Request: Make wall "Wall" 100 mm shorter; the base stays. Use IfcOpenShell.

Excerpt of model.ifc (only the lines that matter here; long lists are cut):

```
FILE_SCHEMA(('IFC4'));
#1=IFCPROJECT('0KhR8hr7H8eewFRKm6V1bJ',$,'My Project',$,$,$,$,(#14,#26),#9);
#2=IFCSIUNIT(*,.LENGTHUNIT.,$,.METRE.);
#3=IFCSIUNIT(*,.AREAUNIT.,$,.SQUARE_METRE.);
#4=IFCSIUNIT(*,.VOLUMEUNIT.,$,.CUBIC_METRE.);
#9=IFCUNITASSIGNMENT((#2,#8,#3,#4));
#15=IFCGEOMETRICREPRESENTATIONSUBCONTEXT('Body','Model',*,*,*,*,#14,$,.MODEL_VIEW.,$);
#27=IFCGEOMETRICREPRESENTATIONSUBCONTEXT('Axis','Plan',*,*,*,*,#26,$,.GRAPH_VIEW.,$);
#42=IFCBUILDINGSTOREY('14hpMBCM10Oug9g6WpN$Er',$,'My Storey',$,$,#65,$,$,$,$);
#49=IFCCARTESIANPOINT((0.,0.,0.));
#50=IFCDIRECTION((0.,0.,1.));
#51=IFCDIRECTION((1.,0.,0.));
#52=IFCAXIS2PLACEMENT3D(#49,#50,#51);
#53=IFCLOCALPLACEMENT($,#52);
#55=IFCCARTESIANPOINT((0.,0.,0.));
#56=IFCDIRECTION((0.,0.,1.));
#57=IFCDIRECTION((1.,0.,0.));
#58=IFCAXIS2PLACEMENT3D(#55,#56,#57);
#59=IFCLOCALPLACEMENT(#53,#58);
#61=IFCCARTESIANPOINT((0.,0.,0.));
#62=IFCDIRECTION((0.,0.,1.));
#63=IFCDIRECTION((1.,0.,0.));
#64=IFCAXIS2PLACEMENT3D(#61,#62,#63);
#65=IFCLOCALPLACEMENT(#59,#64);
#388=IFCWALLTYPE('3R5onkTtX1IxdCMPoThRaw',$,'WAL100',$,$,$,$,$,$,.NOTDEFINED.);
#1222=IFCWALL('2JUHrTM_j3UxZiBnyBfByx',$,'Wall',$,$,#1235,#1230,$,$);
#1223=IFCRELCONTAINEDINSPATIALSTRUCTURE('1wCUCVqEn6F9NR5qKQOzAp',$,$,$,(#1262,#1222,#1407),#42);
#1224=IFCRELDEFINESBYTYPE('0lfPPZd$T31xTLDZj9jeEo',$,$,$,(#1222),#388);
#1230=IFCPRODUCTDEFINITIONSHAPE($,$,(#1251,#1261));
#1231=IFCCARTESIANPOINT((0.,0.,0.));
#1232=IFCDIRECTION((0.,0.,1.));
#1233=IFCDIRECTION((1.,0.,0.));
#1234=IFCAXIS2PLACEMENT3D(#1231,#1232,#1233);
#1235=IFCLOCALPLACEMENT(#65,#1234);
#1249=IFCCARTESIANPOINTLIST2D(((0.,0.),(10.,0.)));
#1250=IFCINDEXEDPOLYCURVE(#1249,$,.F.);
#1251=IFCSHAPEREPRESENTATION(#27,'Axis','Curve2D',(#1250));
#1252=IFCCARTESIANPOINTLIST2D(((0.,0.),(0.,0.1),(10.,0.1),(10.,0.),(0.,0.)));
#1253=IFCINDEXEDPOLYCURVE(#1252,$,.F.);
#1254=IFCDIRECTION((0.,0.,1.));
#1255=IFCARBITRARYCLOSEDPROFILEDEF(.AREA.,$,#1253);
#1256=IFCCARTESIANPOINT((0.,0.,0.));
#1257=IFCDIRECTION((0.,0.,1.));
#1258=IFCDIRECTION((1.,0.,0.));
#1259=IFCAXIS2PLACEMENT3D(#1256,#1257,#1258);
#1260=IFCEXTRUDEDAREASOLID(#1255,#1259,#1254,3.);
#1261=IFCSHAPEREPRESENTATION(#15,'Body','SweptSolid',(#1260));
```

```python
import ifcopenshell
import ifcopenshell.geom
import ifcopenshell.util.representation
import ifcopenshell.util.shape
import ifcopenshell.util.unit

model = ifcopenshell.open("model.ifc")
unit_scale = ifcopenshell.util.unit.calculate_unit_scale(model)
settings = ifcopenshell.geom.settings()


def volume(element):
    """Net volume in cubic metres, openings subtracted."""
    shape = ifcopenshell.geom.create_shape(settings, element)
    return ifcopenshell.util.shape.get_volume(shape.geometry)


wall = model.by_guid("2JUHrTM_j3UxZiBnyBfByx")
before = volume(wall)

body = ifcopenshell.util.representation.get_representation(wall, "Model", "Body")
solid = body.Items[0]
old_height = solid.Depth
solid.Depth -= 0.1 / unit_scale
after = volume(wall)

print(f"height {old_height:g} -> {solid.Depth:g}, volume {before:.3f} -> {after:.3f} m3")

model.write("model_v2.ifc")
```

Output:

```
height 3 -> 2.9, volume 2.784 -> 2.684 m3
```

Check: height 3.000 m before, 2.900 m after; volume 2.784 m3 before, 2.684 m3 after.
